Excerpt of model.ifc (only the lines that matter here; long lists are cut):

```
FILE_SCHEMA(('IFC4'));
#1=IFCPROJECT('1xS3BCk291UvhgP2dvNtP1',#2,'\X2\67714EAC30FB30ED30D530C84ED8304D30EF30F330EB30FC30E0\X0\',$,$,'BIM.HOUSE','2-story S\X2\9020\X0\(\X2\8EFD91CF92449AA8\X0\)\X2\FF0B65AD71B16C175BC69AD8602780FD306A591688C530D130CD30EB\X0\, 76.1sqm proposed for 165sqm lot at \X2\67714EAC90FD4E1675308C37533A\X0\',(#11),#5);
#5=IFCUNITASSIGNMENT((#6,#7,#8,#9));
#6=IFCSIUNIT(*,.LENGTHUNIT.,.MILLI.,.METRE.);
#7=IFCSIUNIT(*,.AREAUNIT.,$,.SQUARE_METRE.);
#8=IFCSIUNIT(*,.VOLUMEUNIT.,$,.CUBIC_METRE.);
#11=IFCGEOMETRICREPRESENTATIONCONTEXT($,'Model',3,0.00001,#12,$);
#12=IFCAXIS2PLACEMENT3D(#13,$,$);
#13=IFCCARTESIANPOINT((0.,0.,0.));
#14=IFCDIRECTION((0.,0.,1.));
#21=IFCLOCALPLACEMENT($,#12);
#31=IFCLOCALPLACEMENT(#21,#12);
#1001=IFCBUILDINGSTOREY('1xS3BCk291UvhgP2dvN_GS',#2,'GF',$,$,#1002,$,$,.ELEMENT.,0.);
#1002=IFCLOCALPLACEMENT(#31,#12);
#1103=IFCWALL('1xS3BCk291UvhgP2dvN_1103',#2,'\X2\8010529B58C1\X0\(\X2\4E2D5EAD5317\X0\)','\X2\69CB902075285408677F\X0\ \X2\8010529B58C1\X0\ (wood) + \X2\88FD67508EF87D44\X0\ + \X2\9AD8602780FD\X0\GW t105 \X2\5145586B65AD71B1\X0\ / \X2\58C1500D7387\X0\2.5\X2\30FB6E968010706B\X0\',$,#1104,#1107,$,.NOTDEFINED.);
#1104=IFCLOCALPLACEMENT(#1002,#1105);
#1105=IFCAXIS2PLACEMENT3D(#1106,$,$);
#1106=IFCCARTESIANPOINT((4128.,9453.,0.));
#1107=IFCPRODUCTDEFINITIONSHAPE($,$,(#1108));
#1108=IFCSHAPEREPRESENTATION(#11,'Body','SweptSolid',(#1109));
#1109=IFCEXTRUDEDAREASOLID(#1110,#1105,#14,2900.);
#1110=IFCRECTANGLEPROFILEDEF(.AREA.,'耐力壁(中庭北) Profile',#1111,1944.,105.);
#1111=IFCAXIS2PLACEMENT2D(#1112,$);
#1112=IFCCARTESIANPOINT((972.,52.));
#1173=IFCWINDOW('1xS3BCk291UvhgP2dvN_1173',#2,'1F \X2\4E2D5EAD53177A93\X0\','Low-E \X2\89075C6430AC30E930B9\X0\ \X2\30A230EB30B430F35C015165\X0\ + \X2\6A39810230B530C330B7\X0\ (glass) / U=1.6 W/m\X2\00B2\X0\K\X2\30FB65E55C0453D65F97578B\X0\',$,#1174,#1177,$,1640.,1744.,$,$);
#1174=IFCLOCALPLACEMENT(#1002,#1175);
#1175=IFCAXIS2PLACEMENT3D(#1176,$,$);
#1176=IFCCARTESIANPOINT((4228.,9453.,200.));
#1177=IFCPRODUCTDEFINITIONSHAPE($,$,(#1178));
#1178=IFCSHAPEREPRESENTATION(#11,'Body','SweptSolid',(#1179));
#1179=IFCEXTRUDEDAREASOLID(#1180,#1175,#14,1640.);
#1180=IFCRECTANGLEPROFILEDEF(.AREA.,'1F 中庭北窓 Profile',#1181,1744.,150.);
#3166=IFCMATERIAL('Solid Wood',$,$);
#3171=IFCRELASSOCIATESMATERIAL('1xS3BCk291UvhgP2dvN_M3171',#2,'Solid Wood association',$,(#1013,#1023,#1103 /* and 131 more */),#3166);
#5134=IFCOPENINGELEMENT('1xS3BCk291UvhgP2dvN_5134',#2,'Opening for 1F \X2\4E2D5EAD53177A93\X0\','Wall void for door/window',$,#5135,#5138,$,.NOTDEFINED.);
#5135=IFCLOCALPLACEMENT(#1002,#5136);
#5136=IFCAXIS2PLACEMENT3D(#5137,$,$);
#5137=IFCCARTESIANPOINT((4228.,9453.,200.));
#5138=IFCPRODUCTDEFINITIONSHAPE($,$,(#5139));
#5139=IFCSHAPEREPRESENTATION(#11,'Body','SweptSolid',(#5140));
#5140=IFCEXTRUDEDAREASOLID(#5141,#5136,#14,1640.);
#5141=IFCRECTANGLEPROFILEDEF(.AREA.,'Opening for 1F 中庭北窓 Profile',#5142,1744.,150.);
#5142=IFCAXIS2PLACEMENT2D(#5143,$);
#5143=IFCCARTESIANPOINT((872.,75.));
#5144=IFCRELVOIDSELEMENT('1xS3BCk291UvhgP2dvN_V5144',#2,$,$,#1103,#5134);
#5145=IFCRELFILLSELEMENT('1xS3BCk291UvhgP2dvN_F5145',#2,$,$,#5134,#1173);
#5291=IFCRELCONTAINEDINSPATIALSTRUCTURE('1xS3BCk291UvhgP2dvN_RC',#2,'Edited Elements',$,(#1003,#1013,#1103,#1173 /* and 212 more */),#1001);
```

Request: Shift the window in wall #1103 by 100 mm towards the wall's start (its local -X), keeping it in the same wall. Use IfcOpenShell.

```python
import ifcopenshell
import ifcopenshell.api.geometry
import ifcopenshell.util.placement
import ifcopenshell.util.unit

model = ifcopenshell.open("model.ifc")
unit_scale = ifcopenshell.util.unit.calculate_unit_scale(model)

window = model.by_guid("1xS3BCk291UvhgP2dvN_1173")
opening = window.FillsVoids[0].RelatingOpeningElement
wall = opening.VoidsElements[0].RelatingBuildingElement

wall_matrix = ifcopenshell.util.placement.get_local_placement(wall.ObjectPlacement)
shift = wall_matrix[:3, 0] * -0.1 / unit_scale
before = ifcopenshell.util.placement.get_local_placement(window.ObjectPlacement)[:3, 3].copy()

# The window is not placed relative to its opening, so move both.
for product in (opening, window):
    matrix = ifcopenshell.util.placement.get_local_placement(product.ObjectPlacement)
    matrix[:3, 3] += shift
    ifcopenshell.api.geometry.edit_object_placement(model, product=product, matrix=matrix, is_si=False)

after = ifcopenshell.util.placement.get_local_placement(window.ObjectPlacement)[:3, 3]
print("window moved by", (after - before).round(3) + 0.0)

model.write("model-out.ifc")
```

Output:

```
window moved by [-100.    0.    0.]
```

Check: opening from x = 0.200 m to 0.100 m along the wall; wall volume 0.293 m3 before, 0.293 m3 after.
